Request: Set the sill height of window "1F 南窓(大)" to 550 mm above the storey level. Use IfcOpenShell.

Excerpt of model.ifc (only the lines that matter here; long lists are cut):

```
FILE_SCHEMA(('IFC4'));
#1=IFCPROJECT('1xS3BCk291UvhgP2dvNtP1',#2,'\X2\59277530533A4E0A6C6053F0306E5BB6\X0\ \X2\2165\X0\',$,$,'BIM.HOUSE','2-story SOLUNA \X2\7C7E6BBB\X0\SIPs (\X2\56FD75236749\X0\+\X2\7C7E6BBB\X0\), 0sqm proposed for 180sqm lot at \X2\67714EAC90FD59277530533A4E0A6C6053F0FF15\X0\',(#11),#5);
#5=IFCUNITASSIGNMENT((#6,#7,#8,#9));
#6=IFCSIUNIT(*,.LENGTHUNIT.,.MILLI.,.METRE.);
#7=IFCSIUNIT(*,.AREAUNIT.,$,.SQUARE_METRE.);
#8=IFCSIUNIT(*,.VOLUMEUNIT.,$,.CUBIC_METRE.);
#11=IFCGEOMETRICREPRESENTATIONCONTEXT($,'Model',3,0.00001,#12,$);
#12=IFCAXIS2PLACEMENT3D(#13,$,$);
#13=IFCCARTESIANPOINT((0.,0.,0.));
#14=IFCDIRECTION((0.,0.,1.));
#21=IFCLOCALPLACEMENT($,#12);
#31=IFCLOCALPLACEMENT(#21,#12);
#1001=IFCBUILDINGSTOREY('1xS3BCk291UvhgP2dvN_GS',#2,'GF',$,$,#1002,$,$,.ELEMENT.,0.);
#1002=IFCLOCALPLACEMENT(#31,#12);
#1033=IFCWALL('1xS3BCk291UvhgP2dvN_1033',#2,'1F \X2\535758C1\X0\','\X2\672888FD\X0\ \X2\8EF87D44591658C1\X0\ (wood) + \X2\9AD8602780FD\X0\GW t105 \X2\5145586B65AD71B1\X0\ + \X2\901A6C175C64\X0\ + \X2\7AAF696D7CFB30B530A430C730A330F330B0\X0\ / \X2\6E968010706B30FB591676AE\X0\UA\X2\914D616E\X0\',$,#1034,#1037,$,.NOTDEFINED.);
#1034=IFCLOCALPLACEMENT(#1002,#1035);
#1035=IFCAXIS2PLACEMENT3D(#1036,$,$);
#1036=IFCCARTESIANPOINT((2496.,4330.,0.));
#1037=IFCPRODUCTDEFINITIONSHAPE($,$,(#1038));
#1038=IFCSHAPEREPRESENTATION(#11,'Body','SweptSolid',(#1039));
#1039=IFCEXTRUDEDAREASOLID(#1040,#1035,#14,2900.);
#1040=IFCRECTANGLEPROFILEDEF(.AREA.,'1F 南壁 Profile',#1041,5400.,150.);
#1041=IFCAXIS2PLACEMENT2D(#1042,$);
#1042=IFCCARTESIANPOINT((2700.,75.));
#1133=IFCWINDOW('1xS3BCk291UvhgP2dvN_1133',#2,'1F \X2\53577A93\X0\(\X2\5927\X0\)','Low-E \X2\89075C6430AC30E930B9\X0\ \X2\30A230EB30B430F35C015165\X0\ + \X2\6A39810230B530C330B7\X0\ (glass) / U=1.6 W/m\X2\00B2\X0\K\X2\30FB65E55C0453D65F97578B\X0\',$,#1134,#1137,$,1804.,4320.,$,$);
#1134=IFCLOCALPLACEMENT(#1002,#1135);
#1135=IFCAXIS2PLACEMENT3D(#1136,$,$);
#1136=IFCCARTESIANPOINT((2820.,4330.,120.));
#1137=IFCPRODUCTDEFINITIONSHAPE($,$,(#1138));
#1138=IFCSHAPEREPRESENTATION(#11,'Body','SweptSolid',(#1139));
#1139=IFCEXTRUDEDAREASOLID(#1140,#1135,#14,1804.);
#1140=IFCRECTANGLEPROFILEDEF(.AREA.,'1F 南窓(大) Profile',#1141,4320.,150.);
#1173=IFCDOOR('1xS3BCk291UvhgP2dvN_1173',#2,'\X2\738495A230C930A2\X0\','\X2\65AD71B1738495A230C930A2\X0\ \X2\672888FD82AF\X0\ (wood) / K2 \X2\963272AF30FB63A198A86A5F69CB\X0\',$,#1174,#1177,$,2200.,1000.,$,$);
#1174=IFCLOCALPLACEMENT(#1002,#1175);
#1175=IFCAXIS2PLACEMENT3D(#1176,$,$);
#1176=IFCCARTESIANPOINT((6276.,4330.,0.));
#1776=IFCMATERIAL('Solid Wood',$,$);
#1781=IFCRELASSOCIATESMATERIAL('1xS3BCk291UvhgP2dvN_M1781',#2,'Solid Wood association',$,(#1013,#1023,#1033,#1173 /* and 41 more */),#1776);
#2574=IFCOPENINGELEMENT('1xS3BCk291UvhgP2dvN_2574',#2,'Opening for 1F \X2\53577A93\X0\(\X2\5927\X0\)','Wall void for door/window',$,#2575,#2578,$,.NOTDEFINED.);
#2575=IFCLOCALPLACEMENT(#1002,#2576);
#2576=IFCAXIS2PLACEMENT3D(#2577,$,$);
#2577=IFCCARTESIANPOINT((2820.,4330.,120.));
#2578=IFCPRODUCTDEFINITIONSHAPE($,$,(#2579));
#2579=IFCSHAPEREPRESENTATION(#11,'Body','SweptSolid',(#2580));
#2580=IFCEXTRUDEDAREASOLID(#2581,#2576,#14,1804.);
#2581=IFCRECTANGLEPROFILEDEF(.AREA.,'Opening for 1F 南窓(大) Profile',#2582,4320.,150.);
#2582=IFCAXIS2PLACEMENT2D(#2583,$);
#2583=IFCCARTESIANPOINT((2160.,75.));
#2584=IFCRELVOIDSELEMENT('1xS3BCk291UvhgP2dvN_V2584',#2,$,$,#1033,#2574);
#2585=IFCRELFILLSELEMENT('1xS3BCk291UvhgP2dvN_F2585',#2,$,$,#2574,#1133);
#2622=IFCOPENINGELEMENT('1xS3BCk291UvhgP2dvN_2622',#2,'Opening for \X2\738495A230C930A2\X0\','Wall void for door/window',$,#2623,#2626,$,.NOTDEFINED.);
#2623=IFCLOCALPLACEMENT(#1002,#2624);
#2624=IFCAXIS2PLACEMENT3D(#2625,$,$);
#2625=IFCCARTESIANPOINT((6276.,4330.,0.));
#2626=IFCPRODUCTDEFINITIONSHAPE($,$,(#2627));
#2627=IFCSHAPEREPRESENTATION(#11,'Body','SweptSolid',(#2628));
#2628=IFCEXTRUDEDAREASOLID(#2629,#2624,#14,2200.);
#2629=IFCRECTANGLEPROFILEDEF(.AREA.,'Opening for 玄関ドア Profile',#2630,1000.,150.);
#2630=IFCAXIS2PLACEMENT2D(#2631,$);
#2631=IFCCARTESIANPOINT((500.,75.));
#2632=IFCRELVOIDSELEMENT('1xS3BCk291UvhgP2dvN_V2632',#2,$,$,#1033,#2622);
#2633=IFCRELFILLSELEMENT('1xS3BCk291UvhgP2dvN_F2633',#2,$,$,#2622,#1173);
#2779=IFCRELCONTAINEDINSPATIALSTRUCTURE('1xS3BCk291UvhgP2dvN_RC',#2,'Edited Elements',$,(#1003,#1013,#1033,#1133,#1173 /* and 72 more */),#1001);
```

```python
import numpy as np
import ifcopenshell
import ifcopenshell.api.geometry
import ifcopenshell.geom
import ifcopenshell.util.element
import ifcopenshell.util.placement
import ifcopenshell.util.shape
import ifcopenshell.util.unit

model = ifcopenshell.open("model.ifc")
unit_scale = ifcopenshell.util.unit.calculate_unit_scale(model)

window = model.by_guid("1xS3BCk291UvhgP2dvN_1133")
opening = window.FillsVoids[0].RelatingOpeningElement
storey = ifcopenshell.util.element.get_container(window, ifc_class="IfcBuildingStorey")
level = ifcopenshell.util.placement.get_local_placement(storey.ObjectPlacement)[2, 3]

# The opening's origin need not be at the sill, so measure its lowest point.
shape = ifcopenshell.geom.create_shape(ifcopenshell.geom.settings(), opening)
bottom = ifcopenshell.util.shape.get_shape_bottom_elevation(shape, shape.geometry) / unit_scale
dz = level + 550.0 - bottom

shift = np.array([0.0, 0.0, dz])
# The window is not placed relative to its opening, so move both.
for product in (opening, window):
    matrix = ifcopenshell.util.placement.get_local_placement(product.ObjectPlacement)
    matrix[:3, 3] += shift
    ifcopenshell.api.geometry.edit_object_placement(model, product=product, matrix=matrix, is_si=False)

print(f"moved by {dz * unit_scale:+.3f} m")

model.write("model-out.ifc")
```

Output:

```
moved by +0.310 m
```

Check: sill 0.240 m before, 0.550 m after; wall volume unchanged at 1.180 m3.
